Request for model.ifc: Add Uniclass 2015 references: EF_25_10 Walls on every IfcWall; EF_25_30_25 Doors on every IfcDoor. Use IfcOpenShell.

First a look at what the model holds.

```python
import ifcopenshell

model = ifcopenshell.open("model.ifc")
print(model.schema)
print("classifications:", [c.Name for c in model.by_type("IfcClassification")])
for ifc_class in ("IfcDoor", "IfcRoof", "IfcStair", "IfcWall", "IfcWindow"):
    print(ifc_class, len(model.by_type(ifc_class)))
```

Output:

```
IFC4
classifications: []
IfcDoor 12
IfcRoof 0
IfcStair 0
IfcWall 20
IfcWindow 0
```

```python
import ifcopenshell
import ifcopenshell.api.classification

model = ifcopenshell.open("model.ifc")

system = ifcopenshell.api.classification.add_classification(model, classification="Uniclass 2015")

codes = {
    "IfcWall": ("EF_25_10", "Walls"),
    "IfcDoor": ("EF_25_30_25", "Doors"),
}
for ifc_class, (code, name) in codes.items():
    products = model.by_type(ifc_class)
    ifcopenshell.api.classification.add_reference(
        model, products=products, classification=system, identification=code, name=name
    )
    print(code, len(products))

model.write("model_v2.ifc")
```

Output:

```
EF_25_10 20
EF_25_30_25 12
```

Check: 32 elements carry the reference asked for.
